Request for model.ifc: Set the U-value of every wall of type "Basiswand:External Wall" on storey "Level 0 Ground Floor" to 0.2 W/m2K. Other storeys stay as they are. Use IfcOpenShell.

First a look at what the model holds.

```python
import ifcopenshell
import ifcopenshell.util.element

model = ifcopenshell.open("model.ifc")
print(model.schema)
storey = next(s for s in model.by_type("IfcBuildingStorey") if s.Name == "Level 0 Ground Floor")
walls = [e for e in ifcopenshell.util.element.get_decomposition(storey) if e.is_a("IfcWall")]
seen = {}
for e in walls:
    element_type = ifcopenshell.util.element.get_type(e)
    key = (element_type.Name if element_type != e and element_type else None, ifcopenshell.util.element.get_pset(e, "Pset_WallCommon", "ThermalTransmittance"))
    seen[key] = seen.get(key, 0) + 1
for (name, value), count in sorted(seen.items(), key=str):
    print(count, "x", name, "|", value)
```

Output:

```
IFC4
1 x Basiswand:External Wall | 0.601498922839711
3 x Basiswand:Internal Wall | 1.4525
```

```python
import ifcopenshell
import ifcopenshell.api.pset
import ifcopenshell.util.element

model = ifcopenshell.open("model.ifc")

storey = next(s for s in model.by_type("IfcBuildingStorey") if s.Name == "Level 0 Ground Floor")
walls = [e for e in ifcopenshell.util.element.get_decomposition(storey) if e.is_a("IfcWall")]

count = 0
for e in walls:
    element_type = ifcopenshell.util.element.get_type(e)
    if element_type in (None, e) or element_type.Name != "Basiswand:External Wall":
        continue
    # add_pset returns the element's existing set when there is one.
    pset = ifcopenshell.api.pset.add_pset(model, product=e, name="Pset_WallCommon")
    ifcopenshell.api.pset.edit_pset(model, pset=pset, properties={"ThermalTransmittance": 0.2})
    count += 1

print(count, "walls updated")

model.write("model_rev.ifc")
```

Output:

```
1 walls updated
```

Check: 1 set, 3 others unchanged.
